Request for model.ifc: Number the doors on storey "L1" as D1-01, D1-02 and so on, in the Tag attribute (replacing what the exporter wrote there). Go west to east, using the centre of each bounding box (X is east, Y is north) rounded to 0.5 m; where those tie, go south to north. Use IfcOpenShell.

First a look at what the model holds.

```python
import ifcopenshell
import ifcopenshell.util.element
import ifcopenshell.util.placement

model = ifcopenshell.open("model.ifc")
print(model.schema)
storey = next(s for s in model.by_type("IfcBuildingStorey") if s.Name == "L1")
doors = [e for e in ifcopenshell.util.element.get_decomposition(storey) if e.is_a("IfcDoor")]
for e in sorted(doors, key=lambda e: e.id()):
    origin = ifcopenshell.util.placement.get_local_placement(e.ObjectPlacement)[:3, 3]
    print(e.id(), e.Tag, e.Name, origin.round(2) + 0.0, sep=" | ")
```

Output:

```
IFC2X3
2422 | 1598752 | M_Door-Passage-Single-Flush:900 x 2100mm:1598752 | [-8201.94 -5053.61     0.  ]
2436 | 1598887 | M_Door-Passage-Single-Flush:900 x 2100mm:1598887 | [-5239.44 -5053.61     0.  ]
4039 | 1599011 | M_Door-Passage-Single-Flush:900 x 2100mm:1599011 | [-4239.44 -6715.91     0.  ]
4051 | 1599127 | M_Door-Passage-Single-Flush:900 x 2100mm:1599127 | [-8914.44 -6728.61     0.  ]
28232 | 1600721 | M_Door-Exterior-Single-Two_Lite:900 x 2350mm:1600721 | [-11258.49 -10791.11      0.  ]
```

```python
import ifcopenshell
import ifcopenshell.geom
import ifcopenshell.util.element
import ifcopenshell.util.shape

model = ifcopenshell.open("model.ifc")
settings = ifcopenshell.geom.settings()
settings.set("use-world-coords", True)


def centre(element):
    shape = ifcopenshell.geom.create_shape(settings, element)
    return ifcopenshell.util.shape.get_bbox_centroid(shape.geometry)


storey = next(s for s in model.by_type("IfcBuildingStorey") if s.Name == "L1")
doors = [e for e in ifcopenshell.util.element.get_decomposition(storey) if e.is_a("IfcDoor")]

# Insertion points can sit at a corner or the storey origin, so sort by the geometry (in metres).
centres = {e: centre(e) for e in doors}
doors.sort(key=lambda e: (round(centres[e][0] / 0.5), centres[e][1]))

for i, e in enumerate(doors, start=1):
    number = f"D1-{i:02d}"
    e.Tag = number
    print(e.id(), number)

model.write("model_edited.ifc")
```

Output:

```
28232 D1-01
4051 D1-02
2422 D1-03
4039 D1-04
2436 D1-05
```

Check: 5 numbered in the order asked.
